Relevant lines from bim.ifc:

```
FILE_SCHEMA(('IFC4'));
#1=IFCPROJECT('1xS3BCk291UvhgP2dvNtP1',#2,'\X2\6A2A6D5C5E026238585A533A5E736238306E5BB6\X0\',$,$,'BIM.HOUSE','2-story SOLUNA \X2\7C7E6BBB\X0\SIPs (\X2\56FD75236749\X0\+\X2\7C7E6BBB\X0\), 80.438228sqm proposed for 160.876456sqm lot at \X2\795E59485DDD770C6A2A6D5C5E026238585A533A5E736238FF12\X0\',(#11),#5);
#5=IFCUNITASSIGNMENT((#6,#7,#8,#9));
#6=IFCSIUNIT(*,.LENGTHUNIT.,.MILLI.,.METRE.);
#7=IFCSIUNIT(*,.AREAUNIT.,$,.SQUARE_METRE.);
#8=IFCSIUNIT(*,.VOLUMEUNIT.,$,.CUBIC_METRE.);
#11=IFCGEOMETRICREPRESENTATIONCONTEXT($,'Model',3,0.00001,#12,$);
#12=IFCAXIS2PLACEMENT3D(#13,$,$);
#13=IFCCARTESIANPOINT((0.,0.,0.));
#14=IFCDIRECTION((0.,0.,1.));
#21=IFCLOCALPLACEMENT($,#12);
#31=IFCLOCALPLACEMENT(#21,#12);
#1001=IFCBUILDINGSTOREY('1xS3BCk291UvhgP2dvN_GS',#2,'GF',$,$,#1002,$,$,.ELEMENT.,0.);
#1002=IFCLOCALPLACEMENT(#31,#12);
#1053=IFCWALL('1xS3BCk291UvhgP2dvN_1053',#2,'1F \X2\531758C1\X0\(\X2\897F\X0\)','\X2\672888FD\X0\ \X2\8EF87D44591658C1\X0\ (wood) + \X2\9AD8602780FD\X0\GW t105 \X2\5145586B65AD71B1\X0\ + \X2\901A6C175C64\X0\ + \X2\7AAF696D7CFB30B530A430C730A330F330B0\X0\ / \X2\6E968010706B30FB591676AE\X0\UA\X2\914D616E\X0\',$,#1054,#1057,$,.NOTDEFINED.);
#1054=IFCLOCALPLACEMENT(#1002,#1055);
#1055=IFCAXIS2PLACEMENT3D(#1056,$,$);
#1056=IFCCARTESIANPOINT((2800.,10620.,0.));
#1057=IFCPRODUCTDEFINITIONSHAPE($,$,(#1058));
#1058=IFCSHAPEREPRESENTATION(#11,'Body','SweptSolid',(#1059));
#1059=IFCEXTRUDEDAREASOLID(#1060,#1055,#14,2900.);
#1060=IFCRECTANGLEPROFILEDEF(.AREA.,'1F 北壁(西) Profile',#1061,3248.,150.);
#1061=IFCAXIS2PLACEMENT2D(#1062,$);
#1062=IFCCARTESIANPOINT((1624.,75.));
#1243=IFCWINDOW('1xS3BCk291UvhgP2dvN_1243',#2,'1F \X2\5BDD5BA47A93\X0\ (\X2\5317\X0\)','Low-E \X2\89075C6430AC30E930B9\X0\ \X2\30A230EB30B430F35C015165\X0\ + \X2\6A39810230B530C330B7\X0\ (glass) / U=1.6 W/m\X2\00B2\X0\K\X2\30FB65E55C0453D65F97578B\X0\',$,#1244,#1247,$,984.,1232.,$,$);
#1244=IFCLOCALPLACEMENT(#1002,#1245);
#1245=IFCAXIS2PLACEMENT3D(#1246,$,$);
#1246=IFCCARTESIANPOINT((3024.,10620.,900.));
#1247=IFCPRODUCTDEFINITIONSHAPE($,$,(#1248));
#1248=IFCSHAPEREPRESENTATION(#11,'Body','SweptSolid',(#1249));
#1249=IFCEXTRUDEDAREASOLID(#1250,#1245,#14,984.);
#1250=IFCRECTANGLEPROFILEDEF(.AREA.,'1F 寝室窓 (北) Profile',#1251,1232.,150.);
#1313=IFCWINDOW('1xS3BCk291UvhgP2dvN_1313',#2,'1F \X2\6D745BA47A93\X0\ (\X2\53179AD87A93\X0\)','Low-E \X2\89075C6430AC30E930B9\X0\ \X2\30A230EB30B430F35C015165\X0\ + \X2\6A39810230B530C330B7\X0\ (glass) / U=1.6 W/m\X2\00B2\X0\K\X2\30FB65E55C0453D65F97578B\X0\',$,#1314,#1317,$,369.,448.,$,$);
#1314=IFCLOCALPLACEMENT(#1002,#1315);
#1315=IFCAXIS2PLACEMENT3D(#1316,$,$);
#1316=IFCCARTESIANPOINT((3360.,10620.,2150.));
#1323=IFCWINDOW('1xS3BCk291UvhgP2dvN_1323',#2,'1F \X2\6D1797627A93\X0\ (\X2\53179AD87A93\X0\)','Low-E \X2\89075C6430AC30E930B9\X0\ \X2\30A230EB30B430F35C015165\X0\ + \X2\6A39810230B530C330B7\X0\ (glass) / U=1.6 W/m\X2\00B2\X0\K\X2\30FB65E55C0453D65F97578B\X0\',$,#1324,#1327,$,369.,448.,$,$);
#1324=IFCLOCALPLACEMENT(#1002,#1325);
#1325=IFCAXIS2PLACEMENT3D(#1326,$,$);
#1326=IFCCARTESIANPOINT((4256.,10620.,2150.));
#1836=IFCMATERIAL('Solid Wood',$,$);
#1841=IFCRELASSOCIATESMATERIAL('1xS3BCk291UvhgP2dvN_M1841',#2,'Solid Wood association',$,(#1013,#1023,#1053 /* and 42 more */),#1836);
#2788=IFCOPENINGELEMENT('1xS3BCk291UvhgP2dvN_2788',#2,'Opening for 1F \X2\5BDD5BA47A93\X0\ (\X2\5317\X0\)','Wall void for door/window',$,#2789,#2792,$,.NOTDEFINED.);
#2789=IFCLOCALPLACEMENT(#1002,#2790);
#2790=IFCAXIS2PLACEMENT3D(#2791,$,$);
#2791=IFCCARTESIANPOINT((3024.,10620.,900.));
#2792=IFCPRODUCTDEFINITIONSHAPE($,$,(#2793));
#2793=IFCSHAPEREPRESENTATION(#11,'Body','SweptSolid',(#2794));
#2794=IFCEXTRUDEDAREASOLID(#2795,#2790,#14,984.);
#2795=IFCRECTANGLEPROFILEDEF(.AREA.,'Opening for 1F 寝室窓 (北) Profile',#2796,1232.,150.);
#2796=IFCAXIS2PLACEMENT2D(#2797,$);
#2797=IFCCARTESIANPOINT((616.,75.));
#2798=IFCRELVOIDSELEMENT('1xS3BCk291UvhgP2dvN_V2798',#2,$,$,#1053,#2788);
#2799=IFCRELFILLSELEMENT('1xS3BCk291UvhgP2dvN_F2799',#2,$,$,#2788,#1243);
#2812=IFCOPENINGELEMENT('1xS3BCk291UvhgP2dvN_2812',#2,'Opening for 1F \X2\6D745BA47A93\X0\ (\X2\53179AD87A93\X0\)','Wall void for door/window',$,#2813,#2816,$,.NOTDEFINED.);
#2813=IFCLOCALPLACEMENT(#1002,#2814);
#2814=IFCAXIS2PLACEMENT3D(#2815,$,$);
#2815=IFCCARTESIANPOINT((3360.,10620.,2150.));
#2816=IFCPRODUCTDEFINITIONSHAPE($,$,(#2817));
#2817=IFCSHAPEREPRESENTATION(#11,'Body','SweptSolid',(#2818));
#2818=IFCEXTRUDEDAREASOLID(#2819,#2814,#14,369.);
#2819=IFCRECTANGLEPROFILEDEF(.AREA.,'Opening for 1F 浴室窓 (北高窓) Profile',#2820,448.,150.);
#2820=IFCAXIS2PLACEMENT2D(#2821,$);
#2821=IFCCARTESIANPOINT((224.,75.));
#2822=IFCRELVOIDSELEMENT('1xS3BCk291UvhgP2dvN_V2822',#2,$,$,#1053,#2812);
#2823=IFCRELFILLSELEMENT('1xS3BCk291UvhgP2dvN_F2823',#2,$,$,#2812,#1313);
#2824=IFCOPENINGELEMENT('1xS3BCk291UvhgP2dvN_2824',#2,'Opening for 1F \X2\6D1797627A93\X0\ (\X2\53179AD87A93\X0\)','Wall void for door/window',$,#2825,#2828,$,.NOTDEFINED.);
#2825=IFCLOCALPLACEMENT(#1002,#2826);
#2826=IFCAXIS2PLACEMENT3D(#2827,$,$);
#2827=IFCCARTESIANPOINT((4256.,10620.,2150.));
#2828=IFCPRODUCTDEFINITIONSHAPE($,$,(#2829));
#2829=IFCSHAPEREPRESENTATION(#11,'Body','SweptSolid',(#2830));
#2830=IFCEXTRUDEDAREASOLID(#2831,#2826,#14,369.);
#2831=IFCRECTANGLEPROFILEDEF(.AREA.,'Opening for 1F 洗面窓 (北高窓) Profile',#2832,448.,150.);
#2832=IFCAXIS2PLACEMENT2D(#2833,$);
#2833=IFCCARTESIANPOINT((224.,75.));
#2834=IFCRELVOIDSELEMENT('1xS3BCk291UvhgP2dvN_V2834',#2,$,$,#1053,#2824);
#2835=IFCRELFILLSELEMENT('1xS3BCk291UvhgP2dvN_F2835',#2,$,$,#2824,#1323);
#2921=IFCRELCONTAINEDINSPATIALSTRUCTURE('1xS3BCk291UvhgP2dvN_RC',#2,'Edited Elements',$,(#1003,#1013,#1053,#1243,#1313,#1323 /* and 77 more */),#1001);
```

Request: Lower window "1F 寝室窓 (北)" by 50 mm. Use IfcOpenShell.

```python
import numpy as np
import ifcopenshell
import ifcopenshell.api.geometry
import ifcopenshell.util.placement
import ifcopenshell.util.unit

model = ifcopenshell.open("bim.ifc")
unit_scale = ifcopenshell.util.unit.calculate_unit_scale(model)

window = model.by_guid("1xS3BCk291UvhgP2dvN_1243")
opening = window.FillsVoids[0].RelatingOpeningElement
dz = -50.0

shift = np.array([0.0, 0.0, dz])
# The window is not placed relative to its opening, so move both.
for product in (opening, window):
    matrix = ifcopenshell.util.placement.get_local_placement(product.ObjectPlacement)
    matrix[:3, 3] += shift
    ifcopenshell.api.geometry.edit_object_placement(model, product=product, matrix=matrix, is_si=False)

print(f"moved by {dz * unit_scale:+.3f} m")

model.write("bim_updated.ifc")
```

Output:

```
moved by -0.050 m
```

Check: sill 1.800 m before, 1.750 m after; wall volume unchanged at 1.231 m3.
